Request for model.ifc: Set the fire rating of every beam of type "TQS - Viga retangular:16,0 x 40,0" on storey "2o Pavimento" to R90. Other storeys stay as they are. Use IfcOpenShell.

First a look at what the model holds.

```python
import ifcopenshell
import ifcopenshell.util.element

model = ifcopenshell.open("model.ifc")
print(model.schema)
storey = next(s for s in model.by_type("IfcBuildingStorey") if s.Name == "2o Pavimento")
beams = [e for e in ifcopenshell.util.element.get_decomposition(storey) if e.is_a("IfcBeam")]
seen = {}
for e in beams:
    element_type = ifcopenshell.util.element.get_type(e)
    key = (element_type.Name if element_type != e and element_type else None, ifcopenshell.util.element.get_pset(e, "Pset_BeamCommon", "FireRating"))
    seen[key] = seen.get(key, 0) + 1
for (name, value), count in sorted(seen.items(), key=str):
    print(count, "x", name, "|", value)
```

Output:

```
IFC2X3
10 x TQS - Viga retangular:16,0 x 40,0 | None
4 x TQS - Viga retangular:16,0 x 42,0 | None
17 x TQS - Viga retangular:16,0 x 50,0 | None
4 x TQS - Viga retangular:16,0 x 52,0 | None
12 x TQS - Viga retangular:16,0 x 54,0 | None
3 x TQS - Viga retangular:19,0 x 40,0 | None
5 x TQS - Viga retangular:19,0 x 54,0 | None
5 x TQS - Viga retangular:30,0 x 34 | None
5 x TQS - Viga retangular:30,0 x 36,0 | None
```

```python
import ifcopenshell
import ifcopenshell.api.pset
import ifcopenshell.util.element

model = ifcopenshell.open("model.ifc")

storey = next(s for s in model.by_type("IfcBuildingStorey") if s.Name == "2o Pavimento")
beams = [e for e in ifcopenshell.util.element.get_decomposition(storey) if e.is_a("IfcBeam")]

count = 0
for e in beams:
    element_type = ifcopenshell.util.element.get_type(e)
    if element_type in (None, e) or element_type.Name != "TQS - Viga retangular:16,0 x 40,0":
        continue
    # add_pset returns the element's existing set when there is one.
    pset = ifcopenshell.api.pset.add_pset(model, product=e, name="Pset_BeamCommon")
    ifcopenshell.api.pset.edit_pset(model, pset=pset, properties={"FireRating": "R90"})
    count += 1

print(count, "beams updated")

model.write("model-out.ifc")
```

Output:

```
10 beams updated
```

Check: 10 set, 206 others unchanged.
